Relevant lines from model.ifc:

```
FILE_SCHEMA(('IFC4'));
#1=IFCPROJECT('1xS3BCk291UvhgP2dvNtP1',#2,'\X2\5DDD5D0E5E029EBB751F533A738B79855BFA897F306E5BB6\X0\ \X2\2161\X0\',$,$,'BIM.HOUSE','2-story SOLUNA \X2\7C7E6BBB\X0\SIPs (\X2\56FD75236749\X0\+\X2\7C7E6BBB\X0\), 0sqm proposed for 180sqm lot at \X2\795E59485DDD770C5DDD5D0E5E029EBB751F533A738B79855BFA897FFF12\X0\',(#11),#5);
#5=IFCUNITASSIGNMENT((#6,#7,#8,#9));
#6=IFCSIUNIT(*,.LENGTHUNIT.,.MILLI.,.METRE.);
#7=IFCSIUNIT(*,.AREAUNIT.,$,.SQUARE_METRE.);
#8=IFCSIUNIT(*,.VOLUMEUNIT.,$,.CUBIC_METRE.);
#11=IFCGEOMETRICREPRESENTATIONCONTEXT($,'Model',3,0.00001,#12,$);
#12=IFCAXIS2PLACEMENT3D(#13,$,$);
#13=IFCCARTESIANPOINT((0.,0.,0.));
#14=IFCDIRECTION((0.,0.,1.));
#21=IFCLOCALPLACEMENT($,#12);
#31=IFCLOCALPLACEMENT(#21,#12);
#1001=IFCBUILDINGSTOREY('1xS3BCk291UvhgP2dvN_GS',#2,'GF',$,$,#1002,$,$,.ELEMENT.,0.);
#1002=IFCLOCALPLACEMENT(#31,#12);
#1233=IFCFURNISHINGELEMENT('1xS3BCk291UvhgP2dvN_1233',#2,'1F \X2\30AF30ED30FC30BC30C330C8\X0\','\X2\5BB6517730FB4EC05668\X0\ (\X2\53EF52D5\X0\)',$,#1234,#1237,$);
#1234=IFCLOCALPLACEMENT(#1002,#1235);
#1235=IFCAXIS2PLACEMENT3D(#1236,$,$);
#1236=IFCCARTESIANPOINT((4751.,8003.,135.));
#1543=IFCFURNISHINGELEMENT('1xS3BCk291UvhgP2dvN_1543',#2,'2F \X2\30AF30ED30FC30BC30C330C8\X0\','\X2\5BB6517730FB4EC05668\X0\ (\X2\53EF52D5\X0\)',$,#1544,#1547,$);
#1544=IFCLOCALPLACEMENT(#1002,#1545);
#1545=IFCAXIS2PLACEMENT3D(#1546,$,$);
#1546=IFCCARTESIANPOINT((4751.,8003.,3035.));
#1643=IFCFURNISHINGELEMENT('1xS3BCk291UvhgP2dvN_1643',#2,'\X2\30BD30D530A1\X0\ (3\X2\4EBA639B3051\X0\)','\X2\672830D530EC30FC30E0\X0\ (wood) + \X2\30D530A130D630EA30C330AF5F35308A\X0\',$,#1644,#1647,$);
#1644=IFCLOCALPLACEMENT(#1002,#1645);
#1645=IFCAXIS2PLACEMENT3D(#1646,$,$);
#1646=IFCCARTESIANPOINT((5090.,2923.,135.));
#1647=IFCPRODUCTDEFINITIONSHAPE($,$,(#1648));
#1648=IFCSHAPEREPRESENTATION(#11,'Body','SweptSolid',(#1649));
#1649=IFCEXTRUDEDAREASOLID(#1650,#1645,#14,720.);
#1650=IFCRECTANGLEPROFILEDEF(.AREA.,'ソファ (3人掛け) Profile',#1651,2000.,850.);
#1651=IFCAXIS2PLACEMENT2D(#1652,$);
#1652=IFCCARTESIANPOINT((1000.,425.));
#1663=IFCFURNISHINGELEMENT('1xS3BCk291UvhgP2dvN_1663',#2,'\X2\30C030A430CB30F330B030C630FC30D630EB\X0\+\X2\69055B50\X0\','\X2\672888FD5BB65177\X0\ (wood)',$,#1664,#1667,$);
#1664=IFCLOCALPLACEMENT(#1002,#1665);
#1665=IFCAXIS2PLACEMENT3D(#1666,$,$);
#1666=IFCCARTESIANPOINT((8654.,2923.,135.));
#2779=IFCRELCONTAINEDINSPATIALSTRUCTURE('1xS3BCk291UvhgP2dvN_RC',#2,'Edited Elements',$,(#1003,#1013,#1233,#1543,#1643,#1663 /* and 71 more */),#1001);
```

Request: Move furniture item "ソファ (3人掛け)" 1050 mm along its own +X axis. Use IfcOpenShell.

```python
import ifcopenshell
import ifcopenshell.api.geometry
import ifcopenshell.util.placement
import ifcopenshell.util.unit

model = ifcopenshell.open("model.ifc")
unit_scale = ifcopenshell.util.unit.calculate_unit_scale(model)

item = model.by_id(1643)
matrix = ifcopenshell.util.placement.get_local_placement(item.ObjectPlacement)
matrix[:3, 3] += matrix[:3, 0] * 1.05 / unit_scale
ifcopenshell.api.geometry.edit_object_placement(model, product=item, matrix=matrix, is_si=False)

print(ifcopenshell.util.placement.get_local_placement(item.ObjectPlacement).round(3) + 0.0)

model.write("model_v2.ifc")
```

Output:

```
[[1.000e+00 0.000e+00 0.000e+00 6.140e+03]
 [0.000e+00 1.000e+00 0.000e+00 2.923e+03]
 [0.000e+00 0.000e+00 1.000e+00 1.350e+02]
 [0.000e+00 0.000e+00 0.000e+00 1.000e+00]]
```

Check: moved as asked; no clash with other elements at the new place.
